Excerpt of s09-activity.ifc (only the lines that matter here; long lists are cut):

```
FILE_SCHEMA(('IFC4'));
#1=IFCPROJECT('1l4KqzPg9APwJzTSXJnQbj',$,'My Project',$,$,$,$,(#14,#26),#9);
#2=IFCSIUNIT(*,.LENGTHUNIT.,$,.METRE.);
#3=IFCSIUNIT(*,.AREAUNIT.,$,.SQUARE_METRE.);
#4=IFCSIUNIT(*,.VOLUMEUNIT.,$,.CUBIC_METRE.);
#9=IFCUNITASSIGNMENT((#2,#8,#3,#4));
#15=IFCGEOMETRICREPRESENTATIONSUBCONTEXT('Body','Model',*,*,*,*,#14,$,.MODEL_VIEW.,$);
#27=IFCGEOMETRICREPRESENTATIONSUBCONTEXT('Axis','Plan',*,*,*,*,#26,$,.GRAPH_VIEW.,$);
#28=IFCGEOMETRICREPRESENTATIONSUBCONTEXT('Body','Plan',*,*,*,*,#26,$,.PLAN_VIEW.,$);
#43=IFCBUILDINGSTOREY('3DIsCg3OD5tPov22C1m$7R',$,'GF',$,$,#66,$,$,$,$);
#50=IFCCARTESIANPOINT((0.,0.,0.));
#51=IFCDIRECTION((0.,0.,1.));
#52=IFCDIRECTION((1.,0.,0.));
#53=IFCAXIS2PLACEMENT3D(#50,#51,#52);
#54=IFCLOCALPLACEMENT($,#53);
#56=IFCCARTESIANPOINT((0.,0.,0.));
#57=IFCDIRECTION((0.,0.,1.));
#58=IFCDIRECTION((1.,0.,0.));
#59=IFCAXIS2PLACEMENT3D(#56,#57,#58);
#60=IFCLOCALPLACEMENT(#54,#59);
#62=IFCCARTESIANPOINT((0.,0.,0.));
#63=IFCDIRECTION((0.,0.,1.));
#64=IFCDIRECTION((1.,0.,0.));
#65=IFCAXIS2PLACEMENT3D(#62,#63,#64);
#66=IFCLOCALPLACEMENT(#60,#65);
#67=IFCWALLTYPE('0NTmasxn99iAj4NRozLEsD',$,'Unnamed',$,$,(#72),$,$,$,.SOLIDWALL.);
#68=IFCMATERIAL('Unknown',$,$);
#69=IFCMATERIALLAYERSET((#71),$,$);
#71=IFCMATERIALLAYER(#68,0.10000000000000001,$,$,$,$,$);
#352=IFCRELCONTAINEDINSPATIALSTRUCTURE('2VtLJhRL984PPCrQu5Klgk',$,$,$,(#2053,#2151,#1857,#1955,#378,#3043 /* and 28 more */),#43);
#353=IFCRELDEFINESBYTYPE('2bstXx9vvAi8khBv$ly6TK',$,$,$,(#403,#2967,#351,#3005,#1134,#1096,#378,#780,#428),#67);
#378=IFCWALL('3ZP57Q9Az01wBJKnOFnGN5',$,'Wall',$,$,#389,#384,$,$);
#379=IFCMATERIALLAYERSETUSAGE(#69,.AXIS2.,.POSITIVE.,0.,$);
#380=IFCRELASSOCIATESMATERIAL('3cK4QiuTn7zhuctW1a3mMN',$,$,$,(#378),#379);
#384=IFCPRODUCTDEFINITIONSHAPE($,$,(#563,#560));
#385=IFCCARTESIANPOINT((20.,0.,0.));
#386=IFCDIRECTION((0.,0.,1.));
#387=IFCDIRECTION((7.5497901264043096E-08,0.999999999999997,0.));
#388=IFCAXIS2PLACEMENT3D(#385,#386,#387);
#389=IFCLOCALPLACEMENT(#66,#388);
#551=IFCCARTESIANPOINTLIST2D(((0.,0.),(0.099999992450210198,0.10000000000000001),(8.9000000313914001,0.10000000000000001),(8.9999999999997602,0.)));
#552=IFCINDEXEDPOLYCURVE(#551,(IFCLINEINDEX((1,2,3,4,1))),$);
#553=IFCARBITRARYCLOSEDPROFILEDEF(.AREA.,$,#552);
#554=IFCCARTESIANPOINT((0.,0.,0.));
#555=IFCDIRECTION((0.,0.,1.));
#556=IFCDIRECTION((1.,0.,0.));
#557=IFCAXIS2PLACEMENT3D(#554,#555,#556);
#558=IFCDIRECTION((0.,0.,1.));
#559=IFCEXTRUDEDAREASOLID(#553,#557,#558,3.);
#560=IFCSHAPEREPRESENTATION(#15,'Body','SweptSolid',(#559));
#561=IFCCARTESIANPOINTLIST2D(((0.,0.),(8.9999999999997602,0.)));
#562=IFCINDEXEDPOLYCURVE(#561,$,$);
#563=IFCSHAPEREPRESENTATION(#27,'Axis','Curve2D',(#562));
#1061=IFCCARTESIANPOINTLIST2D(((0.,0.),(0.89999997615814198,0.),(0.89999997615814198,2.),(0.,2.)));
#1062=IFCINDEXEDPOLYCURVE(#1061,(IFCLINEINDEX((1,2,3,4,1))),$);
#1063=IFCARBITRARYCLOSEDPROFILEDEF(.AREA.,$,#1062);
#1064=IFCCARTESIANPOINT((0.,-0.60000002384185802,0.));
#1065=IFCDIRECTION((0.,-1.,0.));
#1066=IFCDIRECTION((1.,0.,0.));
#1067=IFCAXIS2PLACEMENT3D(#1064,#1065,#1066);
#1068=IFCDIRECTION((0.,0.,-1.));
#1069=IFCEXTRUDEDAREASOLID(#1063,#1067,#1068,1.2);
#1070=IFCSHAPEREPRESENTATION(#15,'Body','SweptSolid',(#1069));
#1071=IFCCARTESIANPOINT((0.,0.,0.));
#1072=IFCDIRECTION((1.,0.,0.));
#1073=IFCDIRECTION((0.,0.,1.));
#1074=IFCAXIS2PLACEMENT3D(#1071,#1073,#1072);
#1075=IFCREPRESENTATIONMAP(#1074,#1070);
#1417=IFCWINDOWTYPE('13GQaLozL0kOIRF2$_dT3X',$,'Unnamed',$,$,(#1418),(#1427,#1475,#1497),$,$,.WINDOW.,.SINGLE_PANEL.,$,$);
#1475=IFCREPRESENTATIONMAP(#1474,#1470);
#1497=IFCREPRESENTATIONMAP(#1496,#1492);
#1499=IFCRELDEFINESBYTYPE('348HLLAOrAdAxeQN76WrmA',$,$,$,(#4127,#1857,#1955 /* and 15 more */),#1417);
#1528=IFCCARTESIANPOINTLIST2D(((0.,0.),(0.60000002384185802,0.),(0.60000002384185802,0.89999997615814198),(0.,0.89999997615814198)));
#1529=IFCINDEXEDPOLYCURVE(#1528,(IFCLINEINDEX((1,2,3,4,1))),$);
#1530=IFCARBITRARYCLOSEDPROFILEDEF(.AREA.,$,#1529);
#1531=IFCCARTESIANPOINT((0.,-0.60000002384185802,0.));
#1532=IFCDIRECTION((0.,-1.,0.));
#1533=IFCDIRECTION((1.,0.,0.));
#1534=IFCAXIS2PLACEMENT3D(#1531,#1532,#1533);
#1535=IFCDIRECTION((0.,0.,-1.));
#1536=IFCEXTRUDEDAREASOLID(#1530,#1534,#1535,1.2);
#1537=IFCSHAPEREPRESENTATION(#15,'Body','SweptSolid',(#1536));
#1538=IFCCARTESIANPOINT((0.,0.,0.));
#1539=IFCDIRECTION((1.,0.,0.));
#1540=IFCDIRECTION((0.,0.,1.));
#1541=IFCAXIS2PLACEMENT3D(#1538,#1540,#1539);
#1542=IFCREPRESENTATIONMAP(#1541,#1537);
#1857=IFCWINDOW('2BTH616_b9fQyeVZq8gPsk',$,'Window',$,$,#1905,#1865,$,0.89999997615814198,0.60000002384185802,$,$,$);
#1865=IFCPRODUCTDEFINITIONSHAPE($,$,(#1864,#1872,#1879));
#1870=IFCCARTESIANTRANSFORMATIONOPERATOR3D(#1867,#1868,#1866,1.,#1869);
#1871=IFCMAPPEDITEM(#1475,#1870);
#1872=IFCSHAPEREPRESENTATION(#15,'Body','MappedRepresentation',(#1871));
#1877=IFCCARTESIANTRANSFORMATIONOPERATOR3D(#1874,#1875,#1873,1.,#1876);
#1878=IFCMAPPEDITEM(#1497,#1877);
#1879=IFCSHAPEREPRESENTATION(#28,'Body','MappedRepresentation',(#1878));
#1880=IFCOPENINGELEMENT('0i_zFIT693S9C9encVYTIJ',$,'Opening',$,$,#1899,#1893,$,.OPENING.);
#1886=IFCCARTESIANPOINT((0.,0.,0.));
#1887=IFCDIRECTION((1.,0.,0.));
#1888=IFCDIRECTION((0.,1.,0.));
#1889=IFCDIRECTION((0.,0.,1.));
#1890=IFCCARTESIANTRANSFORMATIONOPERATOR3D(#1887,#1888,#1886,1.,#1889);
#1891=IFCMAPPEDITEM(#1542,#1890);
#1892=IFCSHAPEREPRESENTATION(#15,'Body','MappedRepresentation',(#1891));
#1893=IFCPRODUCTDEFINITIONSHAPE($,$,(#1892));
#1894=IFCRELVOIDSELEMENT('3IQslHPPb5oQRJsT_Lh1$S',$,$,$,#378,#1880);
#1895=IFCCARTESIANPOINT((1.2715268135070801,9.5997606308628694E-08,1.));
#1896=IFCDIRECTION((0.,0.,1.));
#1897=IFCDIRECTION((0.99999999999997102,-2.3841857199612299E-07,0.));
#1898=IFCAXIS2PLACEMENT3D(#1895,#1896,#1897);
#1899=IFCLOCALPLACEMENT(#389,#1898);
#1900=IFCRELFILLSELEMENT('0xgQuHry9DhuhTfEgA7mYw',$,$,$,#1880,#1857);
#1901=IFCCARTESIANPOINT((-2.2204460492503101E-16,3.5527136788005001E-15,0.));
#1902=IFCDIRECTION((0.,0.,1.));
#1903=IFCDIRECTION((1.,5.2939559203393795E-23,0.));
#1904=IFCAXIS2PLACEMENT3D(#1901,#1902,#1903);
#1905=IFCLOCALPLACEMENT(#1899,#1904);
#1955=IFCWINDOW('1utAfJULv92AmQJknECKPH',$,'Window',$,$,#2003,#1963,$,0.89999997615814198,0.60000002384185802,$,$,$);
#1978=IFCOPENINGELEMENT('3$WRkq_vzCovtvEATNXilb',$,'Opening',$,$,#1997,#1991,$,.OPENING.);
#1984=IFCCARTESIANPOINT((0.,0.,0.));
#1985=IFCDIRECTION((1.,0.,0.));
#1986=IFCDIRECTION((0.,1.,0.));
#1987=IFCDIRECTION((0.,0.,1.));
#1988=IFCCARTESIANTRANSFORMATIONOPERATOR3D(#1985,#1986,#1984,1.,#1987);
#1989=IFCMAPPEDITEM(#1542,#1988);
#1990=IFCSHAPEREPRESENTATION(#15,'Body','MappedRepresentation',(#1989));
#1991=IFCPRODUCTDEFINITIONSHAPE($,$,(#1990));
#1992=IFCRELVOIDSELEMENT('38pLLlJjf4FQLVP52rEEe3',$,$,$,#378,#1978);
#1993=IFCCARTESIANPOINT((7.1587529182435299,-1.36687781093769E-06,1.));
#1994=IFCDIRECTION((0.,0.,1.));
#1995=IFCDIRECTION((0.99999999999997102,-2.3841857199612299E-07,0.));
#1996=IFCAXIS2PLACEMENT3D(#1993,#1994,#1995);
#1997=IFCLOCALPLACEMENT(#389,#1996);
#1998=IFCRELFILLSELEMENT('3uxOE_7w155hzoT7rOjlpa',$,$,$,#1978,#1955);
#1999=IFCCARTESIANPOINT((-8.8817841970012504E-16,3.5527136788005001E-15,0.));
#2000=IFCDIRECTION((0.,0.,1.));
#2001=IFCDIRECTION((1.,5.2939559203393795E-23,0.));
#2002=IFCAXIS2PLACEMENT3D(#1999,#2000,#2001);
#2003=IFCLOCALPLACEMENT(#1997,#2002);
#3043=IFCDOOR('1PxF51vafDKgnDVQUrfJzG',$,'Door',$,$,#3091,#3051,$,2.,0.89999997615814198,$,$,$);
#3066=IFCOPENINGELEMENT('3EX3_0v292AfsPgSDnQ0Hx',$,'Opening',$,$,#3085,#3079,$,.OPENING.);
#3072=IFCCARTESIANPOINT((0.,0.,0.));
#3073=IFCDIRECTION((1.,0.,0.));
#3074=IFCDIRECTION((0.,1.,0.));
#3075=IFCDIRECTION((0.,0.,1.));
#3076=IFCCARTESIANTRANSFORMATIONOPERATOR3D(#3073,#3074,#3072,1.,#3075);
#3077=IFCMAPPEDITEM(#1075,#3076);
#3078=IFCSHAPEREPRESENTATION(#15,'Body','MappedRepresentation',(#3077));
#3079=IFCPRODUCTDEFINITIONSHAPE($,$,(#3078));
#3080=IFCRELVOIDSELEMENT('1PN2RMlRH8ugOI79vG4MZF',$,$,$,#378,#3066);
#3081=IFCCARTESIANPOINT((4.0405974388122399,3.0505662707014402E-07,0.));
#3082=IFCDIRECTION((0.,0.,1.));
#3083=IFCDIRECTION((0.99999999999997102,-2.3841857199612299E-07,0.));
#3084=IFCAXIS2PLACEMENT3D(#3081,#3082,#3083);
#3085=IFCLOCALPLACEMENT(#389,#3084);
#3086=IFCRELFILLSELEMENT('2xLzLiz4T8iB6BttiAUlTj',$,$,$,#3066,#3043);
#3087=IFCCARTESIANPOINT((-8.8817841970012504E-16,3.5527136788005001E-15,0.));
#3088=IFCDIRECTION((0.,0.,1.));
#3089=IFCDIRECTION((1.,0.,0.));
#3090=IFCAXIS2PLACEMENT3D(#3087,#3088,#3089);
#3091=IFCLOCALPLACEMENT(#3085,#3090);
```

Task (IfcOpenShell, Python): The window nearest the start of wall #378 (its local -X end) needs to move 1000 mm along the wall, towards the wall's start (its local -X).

```python
import ifcopenshell
import ifcopenshell.api.geometry
import ifcopenshell.util.placement
import ifcopenshell.util.unit

model = ifcopenshell.open("s09-activity.ifc")
unit_scale = ifcopenshell.util.unit.calculate_unit_scale(model)

window = model.by_id(1857)
opening = window.FillsVoids[0].RelatingOpeningElement
wall = opening.VoidsElements[0].RelatingBuildingElement

wall_matrix = ifcopenshell.util.placement.get_local_placement(wall.ObjectPlacement)
shift = wall_matrix[:3, 0] * -1 / unit_scale
before = ifcopenshell.util.placement.get_local_placement(window.ObjectPlacement)[:3, 3].copy()

# The window is placed relative to its opening, so it follows when the opening moves.
matrix = ifcopenshell.util.placement.get_local_placement(opening.ObjectPlacement)
matrix[:3, 3] += shift
ifcopenshell.api.geometry.edit_object_placement(
    model, product=opening, matrix=matrix, is_si=False, should_transform_children=True
)

after = ifcopenshell.util.placement.get_local_placement(window.ObjectPlacement)[:3, 3]
print("window moved by", (after - before).round(3) + 0.0)

model.write("s09-activity_rev.ifc")
```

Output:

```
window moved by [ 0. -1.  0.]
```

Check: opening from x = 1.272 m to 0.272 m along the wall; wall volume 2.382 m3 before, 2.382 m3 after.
